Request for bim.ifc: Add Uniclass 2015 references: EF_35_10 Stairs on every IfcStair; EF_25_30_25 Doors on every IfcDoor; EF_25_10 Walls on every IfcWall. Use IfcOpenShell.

First a look at what the model holds.

```python
import ifcopenshell

model = ifcopenshell.open("bim.ifc")
print(model.schema)
print("classifications:", [c.Name for c in model.by_type("IfcClassification")])
for ifc_class in ("IfcDoor", "IfcRoof", "IfcStair", "IfcWall", "IfcWindow"):
    print(ifc_class, len(model.by_type(ifc_class)))
```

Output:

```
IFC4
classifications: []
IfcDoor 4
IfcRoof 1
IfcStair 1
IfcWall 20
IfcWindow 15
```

```python
import ifcopenshell
import ifcopenshell.api.classification

model = ifcopenshell.open("bim.ifc")

system = ifcopenshell.api.classification.add_classification(model, classification="Uniclass 2015")

codes = {
    "IfcStair": ("EF_35_10", "Stairs"),
    "IfcDoor": ("EF_25_30_25", "Doors"),
    "IfcWall": ("EF_25_10", "Walls"),
}
for ifc_class, (code, name) in codes.items():
    products = model.by_type(ifc_class)
    ifcopenshell.api.classification.add_reference(
        model, products=products, classification=system, identification=code, name=name
    )
    print(code, len(products))

model.write("bim_rev.ifc")
```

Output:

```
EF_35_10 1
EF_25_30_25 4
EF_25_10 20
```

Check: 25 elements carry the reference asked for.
